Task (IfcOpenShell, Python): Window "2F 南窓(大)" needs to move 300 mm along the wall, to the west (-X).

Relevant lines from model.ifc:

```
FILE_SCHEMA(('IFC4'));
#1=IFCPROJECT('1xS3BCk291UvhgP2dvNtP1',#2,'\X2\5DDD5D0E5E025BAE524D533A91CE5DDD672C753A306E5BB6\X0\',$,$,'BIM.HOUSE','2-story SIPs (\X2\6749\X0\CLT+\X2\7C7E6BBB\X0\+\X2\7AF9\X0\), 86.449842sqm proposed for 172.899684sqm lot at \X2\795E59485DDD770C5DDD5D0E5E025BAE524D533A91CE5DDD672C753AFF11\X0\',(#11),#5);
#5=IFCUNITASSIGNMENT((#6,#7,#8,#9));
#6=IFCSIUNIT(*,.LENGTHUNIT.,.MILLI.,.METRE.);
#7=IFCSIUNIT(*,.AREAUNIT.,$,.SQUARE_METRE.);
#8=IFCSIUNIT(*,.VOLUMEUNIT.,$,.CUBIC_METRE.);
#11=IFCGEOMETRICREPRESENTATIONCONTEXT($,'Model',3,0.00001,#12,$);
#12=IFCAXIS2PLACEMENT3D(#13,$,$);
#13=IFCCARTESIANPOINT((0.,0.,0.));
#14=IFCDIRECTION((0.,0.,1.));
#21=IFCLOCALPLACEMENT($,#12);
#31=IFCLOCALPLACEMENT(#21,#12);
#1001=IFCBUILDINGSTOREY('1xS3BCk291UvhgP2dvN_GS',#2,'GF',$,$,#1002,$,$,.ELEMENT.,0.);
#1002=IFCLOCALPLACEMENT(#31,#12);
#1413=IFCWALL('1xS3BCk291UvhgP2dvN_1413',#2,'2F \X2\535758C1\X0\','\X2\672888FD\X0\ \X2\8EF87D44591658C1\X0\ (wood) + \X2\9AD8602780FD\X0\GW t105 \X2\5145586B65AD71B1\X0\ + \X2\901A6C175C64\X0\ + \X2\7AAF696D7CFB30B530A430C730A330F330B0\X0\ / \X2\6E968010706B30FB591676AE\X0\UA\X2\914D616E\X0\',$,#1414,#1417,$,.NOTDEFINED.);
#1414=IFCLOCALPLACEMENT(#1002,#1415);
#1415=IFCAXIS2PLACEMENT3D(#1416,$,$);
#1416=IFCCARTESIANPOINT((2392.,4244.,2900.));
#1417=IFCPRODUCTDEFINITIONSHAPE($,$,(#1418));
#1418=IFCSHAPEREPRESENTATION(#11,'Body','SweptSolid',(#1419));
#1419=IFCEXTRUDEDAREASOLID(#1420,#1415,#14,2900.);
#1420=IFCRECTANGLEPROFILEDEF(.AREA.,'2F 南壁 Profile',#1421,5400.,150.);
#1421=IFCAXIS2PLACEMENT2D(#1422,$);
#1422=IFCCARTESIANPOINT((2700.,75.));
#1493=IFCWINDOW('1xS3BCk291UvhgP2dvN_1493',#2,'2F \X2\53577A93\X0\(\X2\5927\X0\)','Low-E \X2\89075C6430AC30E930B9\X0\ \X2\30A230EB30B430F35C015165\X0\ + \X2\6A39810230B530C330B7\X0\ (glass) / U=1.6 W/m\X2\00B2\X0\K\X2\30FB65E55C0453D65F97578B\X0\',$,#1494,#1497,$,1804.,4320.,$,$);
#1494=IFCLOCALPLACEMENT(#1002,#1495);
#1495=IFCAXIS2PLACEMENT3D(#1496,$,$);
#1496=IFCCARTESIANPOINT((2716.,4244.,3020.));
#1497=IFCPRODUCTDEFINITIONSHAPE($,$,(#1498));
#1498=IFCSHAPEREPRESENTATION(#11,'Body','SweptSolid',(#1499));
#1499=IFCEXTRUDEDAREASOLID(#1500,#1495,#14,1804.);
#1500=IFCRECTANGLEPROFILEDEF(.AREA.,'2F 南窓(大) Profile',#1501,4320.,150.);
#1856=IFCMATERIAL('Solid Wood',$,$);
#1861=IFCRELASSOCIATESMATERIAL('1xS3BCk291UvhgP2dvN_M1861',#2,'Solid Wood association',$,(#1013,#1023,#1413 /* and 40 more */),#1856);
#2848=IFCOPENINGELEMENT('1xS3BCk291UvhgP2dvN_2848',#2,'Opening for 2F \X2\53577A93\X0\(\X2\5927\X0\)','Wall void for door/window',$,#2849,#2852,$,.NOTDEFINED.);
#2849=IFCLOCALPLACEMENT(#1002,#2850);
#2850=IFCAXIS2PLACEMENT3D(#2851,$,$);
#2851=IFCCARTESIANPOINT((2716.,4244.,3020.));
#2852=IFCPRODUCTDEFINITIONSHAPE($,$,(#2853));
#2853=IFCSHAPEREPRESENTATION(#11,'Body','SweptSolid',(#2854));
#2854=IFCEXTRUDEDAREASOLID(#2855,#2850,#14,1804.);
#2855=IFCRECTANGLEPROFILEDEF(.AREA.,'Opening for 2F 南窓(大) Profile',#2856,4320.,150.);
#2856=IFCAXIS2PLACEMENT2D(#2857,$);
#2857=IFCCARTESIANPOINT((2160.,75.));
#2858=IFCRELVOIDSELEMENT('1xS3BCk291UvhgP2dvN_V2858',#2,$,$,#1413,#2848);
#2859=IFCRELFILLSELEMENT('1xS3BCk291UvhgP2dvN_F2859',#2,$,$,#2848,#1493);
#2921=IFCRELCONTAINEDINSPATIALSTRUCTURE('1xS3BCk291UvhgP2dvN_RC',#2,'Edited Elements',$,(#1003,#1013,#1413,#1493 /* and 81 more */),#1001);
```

```python
import ifcopenshell
import ifcopenshell.api.geometry
import ifcopenshell.util.placement
import ifcopenshell.util.unit

model = ifcopenshell.open("model.ifc")
unit_scale = ifcopenshell.util.unit.calculate_unit_scale(model)

window = model.by_id(1493)
opening = window.FillsVoids[0].RelatingOpeningElement
wall = opening.VoidsElements[0].RelatingBuildingElement

wall_matrix = ifcopenshell.util.placement.get_local_placement(wall.ObjectPlacement)
shift = wall_matrix[:3, 0] * -0.3 / unit_scale
before = ifcopenshell.util.placement.get_local_placement(window.ObjectPlacement)[:3, 3].copy()

# The window is not placed relative to its opening, so move both.
for product in (opening, window):
    matrix = ifcopenshell.util.placement.get_local_placement(product.ObjectPlacement)
    matrix[:3, 3] += shift
    ifcopenshell.api.geometry.edit_object_placement(model, product=product, matrix=matrix, is_si=False)

after = ifcopenshell.util.placement.get_local_placement(window.ObjectPlacement)[:3, 3]
print("window moved by", (after - before).round(3) + 0.0)

model.write("model_edited.ifc")
```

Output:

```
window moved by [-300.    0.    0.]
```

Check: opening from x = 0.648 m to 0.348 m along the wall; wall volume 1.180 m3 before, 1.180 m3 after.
